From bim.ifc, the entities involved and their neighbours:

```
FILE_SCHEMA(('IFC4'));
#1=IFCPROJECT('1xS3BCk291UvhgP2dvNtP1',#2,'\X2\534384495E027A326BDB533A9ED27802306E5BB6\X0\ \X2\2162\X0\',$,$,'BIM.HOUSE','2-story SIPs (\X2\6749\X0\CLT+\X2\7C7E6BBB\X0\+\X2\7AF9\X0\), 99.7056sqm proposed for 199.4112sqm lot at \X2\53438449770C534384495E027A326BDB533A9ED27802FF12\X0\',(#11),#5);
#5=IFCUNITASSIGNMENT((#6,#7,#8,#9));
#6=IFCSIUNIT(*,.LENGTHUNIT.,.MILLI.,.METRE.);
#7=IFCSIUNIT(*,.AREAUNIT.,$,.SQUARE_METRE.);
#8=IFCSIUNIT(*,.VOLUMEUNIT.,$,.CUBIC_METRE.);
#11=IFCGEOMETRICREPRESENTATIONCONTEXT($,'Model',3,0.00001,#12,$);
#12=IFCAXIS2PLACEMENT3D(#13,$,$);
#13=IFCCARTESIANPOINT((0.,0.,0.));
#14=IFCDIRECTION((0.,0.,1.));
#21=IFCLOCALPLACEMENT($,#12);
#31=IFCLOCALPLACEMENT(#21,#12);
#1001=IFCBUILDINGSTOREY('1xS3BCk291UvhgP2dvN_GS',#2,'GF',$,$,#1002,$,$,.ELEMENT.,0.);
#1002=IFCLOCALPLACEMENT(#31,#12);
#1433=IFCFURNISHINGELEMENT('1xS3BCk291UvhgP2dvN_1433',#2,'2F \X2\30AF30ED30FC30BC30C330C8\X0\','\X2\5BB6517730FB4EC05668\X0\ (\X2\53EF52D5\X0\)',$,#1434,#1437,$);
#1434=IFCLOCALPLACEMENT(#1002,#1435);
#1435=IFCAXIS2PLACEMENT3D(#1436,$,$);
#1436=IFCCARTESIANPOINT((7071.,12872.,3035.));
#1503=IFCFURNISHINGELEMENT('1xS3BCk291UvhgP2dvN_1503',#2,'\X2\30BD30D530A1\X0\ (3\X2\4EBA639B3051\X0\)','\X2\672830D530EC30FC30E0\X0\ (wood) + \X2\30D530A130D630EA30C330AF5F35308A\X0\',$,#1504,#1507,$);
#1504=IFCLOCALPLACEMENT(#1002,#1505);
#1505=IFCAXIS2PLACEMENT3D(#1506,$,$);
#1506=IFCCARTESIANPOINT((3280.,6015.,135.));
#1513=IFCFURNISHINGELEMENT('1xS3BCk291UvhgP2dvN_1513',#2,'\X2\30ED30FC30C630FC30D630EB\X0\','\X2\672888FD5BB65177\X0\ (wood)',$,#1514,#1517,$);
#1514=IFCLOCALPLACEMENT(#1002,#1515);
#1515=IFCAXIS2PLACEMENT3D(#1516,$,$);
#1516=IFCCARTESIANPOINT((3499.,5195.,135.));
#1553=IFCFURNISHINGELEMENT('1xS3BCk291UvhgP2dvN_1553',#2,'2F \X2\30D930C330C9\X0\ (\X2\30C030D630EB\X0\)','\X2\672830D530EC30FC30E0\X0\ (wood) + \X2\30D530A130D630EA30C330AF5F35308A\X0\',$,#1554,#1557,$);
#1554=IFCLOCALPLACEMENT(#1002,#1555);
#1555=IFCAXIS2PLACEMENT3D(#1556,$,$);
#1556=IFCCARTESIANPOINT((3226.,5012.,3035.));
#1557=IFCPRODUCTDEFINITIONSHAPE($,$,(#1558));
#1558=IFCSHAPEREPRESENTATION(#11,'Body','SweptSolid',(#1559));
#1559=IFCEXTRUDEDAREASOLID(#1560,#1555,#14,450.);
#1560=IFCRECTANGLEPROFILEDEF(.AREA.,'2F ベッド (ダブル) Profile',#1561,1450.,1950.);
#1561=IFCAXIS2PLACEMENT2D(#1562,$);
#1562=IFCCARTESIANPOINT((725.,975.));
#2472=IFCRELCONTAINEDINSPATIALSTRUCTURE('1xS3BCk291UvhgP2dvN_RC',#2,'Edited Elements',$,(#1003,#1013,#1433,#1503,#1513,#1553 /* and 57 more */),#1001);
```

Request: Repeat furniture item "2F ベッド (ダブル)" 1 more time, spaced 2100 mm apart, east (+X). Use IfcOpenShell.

```python
import numpy as np
import ifcopenshell
import ifcopenshell.api.geometry
import ifcopenshell.api.root
import ifcopenshell.util.element
import ifcopenshell.util.placement
import ifcopenshell.util.unit

model = ifcopenshell.open("bim.ifc")
unit_scale = ifcopenshell.util.unit.calculate_unit_scale(model)


def reuse_history(source, copy):
    """copy_class also copies each property set's owner history, people and application; keep the originals."""
    for rel in copy.IsDefinedBy:
        if rel.is_a("IfcRelDefinesByProperties") and (history := rel.RelatingPropertyDefinition.OwnerHistory):
            rel.RelatingPropertyDefinition.OwnerHistory = source.OwnerHistory
            ifcopenshell.util.element.remove_deep2(model, history)


source = model.by_guid("1xS3BCk291UvhgP2dvN_1553")
base = ifcopenshell.util.placement.get_local_placement(source.ObjectPlacement)
step = np.array([1.0, 0.0, 0.0]) * 2.1 / unit_scale

for i in range(1, 2):
    copy = ifcopenshell.api.root.copy_class(model, product=source)
    copy.Representation = ifcopenshell.util.element.copy_deep(
        model, source.Representation, exclude=["IfcGeometricRepresentationContext", "IfcRepresentationMap"]
    )
    reuse_history(source, copy)
    matrix = base.copy()
    matrix[:3, 3] += i * step
    print("added at", matrix[:3, 3].round(3) + 0.0)
    ifcopenshell.api.geometry.edit_object_placement(model, product=copy, matrix=matrix, is_si=False)

model.write("bim_rev.ifc")
```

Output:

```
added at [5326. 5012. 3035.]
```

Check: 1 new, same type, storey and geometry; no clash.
